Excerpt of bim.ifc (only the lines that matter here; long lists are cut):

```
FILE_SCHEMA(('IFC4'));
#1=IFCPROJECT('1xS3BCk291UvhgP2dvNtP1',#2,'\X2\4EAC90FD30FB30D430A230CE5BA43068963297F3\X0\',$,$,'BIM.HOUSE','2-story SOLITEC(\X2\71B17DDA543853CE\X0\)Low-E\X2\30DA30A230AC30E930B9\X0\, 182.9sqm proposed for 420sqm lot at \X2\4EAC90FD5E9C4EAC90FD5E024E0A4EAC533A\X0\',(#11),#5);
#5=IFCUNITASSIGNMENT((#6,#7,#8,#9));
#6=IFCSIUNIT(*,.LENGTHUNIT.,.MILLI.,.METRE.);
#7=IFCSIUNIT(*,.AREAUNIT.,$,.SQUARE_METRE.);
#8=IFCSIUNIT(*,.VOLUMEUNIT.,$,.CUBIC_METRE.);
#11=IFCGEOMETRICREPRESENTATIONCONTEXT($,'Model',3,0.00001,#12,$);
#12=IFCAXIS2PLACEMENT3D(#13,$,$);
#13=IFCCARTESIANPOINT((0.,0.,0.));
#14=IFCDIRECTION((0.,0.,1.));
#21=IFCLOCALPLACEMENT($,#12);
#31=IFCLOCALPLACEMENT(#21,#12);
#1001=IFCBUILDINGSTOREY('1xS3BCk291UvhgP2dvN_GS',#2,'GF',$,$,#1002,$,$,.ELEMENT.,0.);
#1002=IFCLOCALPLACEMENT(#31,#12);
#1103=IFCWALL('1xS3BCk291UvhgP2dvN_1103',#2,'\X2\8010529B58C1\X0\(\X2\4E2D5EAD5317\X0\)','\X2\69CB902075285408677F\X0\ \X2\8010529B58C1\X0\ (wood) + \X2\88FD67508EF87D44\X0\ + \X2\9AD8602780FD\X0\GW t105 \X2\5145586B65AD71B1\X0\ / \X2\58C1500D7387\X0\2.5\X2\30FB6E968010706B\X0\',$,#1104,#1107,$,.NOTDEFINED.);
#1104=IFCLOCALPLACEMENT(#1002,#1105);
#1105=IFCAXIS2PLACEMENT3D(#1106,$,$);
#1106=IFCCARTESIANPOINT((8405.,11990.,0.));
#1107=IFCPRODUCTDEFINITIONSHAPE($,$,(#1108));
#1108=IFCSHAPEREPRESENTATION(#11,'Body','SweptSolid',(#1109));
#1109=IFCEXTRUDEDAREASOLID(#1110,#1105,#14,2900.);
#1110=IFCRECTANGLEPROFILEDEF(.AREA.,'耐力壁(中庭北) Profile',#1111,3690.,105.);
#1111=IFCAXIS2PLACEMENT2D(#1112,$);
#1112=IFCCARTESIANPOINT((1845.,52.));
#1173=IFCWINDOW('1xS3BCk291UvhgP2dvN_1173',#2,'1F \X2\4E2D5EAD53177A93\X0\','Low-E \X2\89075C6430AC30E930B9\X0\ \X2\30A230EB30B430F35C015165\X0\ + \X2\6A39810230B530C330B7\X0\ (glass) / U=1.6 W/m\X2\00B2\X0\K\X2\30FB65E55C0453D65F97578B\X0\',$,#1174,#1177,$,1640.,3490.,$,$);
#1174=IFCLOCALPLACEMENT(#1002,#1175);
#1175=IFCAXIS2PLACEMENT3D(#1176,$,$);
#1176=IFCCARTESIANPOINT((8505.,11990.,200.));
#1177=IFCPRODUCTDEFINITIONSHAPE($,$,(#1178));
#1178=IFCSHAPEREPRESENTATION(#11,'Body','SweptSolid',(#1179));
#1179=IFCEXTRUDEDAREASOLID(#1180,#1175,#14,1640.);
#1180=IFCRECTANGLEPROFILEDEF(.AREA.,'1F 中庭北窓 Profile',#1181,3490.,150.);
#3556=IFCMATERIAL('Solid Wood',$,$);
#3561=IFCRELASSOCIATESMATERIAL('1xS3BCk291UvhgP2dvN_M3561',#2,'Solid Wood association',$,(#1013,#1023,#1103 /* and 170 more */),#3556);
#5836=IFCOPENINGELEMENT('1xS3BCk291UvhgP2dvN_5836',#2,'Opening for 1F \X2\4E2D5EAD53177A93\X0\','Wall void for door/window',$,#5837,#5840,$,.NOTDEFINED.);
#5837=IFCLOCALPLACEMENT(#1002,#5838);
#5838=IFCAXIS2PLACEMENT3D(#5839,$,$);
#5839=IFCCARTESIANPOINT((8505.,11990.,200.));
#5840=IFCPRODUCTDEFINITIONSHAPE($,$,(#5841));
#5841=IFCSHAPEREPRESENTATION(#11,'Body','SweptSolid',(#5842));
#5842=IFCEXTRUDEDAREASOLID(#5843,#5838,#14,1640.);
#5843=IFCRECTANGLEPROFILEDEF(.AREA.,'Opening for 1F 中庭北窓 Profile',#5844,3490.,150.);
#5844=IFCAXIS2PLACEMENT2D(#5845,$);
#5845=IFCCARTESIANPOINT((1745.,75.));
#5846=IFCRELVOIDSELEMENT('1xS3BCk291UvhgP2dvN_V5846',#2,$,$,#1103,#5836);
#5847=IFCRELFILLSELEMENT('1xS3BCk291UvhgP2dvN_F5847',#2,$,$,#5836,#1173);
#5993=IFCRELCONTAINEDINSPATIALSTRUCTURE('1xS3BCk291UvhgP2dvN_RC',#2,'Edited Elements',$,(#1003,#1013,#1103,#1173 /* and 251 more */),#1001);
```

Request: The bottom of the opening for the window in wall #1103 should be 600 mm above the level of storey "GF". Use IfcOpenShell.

```python
import numpy as np
import ifcopenshell
import ifcopenshell.api.geometry
import ifcopenshell.geom
import ifcopenshell.util.element
import ifcopenshell.util.placement
import ifcopenshell.util.shape
import ifcopenshell.util.unit

model = ifcopenshell.open("bim.ifc")
unit_scale = ifcopenshell.util.unit.calculate_unit_scale(model)

window = model.by_guid("1xS3BCk291UvhgP2dvN_1173")
opening = window.FillsVoids[0].RelatingOpeningElement
storey = ifcopenshell.util.element.get_container(window, ifc_class="IfcBuildingStorey")
level = ifcopenshell.util.placement.get_local_placement(storey.ObjectPlacement)[2, 3]

# The opening's origin need not be at the sill, so measure its lowest point.
shape = ifcopenshell.geom.create_shape(ifcopenshell.geom.settings(), opening)
bottom = ifcopenshell.util.shape.get_shape_bottom_elevation(shape, shape.geometry) / unit_scale
dz = level + 600.0 - bottom

shift = np.array([0.0, 0.0, dz])
# The window is not placed relative to its opening, so move both.
for product in (opening, window):
    matrix = ifcopenshell.util.placement.get_local_placement(product.ObjectPlacement)
    matrix[:3, 3] += shift
    ifcopenshell.api.geometry.edit_object_placement(model, product=product, matrix=matrix, is_si=False)

print(f"moved by {dz * unit_scale:+.3f} m")

model.write("bim_updated.ifc")
```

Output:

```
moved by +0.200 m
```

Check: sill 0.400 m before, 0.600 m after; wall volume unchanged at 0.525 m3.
